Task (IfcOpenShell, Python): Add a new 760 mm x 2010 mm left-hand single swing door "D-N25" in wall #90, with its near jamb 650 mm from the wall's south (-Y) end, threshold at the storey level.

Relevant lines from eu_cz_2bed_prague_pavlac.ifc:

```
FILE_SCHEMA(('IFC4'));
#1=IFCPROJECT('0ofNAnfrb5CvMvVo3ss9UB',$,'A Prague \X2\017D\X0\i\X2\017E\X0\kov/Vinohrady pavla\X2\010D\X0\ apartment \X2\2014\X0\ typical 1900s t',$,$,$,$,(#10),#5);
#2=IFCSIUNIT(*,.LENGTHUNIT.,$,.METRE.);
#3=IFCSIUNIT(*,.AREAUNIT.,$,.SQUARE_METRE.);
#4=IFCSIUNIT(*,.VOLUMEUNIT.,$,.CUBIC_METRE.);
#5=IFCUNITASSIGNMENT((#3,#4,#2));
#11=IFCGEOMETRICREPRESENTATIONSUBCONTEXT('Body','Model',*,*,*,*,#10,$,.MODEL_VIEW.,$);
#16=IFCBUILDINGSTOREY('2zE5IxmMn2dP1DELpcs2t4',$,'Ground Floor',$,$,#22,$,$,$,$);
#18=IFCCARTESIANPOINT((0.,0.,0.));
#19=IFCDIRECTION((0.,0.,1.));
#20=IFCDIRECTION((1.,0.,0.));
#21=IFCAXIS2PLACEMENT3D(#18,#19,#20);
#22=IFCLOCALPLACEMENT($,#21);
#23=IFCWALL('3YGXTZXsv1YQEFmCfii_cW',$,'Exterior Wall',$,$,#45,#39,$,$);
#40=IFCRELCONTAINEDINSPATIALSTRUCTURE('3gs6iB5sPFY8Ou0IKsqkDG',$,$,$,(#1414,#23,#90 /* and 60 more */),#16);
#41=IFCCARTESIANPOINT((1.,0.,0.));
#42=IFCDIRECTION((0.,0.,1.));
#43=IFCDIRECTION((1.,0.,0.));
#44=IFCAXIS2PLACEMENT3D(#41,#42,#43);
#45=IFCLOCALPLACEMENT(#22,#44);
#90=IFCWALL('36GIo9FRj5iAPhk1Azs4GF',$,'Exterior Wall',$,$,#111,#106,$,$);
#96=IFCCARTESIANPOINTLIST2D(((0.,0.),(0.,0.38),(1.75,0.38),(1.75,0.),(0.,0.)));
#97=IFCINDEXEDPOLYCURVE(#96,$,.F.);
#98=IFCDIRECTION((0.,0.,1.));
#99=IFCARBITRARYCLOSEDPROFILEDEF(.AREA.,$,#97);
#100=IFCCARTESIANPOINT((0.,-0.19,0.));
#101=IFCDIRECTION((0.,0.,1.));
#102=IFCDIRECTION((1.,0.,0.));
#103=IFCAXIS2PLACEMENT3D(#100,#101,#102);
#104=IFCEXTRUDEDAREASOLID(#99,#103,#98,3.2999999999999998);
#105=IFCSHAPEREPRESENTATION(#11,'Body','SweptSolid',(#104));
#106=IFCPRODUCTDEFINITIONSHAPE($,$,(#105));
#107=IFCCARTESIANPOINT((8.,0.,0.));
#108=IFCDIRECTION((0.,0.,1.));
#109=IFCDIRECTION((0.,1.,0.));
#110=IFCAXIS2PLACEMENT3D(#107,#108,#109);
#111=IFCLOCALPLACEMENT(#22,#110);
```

```python
import numpy as np
import ifcopenshell
import ifcopenshell.api.feature
import ifcopenshell.api.geometry
import ifcopenshell.api.root
import ifcopenshell.api.spatial
import ifcopenshell.geom
import ifcopenshell.util.element
import ifcopenshell.util.placement
import ifcopenshell.util.representation
import ifcopenshell.util.shape
import ifcopenshell.util.unit

model = ifcopenshell.open("eu_cz_2bed_prague_pavlac.ifc")
unit_scale = ifcopenshell.util.unit.calculate_unit_scale(model)
settings = ifcopenshell.geom.settings()


def volume(element):
    """Net volume in cubic metres, openings subtracted."""
    shape = ifcopenshell.geom.create_shape(settings, element)
    return ifcopenshell.util.shape.get_volume(shape.geometry)


wall = model.by_guid("36GIo9FRj5iAPhk1Azs4GF")
storey = ifcopenshell.util.element.get_container(wall, ifc_class="IfcBuildingStorey")
context = ifcopenshell.util.representation.get_context(model, "Model", "Body", "MODEL_VIEW")
before = volume(wall)

width, height, from_end, sill = 0.76, 2.01, 0.65, 0.0  # metres

# The wall runs along its own X axis, and the end named is its -X end.
wall_shape = ifcopenshell.geom.create_shape(settings, wall)
x, y, z = ifcopenshell.util.shape.get_vertices(wall_shape.geometry).T
start = x.min() + from_end
face, thickness = float(y.min()), float(y.max() - y.min())
wall_matrix = ifcopenshell.util.placement.get_local_placement(wall.ObjectPlacement)
level = ifcopenshell.util.placement.get_local_placement(storey.ObjectPlacement)[2, 3]


def in_wall(x, y):
    """Placement at x, y metres in the wall's axes, at sill height."""
    matrix = wall_matrix.copy()
    matrix[:, 3] = wall_matrix @ np.array([x / unit_scale, y / unit_scale, 0.0, 1.0])
    matrix[2, 3] = level + sill / unit_scale
    return matrix


# Opening: a box that overshoots both wall faces by 50 mm.
opening = ifcopenshell.api.root.create_entity(model, ifc_class="IfcOpeningElement", predefined_type="OPENING")
box = ifcopenshell.api.geometry.add_wall_representation(
    model, context=context, length=width, height=height, thickness=thickness + 0.1
)
ifcopenshell.api.geometry.assign_representation(model, product=opening, representation=box)
ifcopenshell.api.geometry.edit_object_placement(model, product=opening, matrix=in_wall(start, face - 0.05), is_si=False)
ifcopenshell.api.feature.add_feature(model, feature=opening, element=wall)

door = ifcopenshell.api.root.create_entity(model, ifc_class="IfcDoor", name="D-N25", predefined_type="DOOR")
door.OverallWidth, door.OverallHeight = width / unit_scale, height / unit_scale
door.OperationType = "SINGLE_SWING_LEFT"
body = ifcopenshell.api.geometry.add_door_representation(
    model,
    context=context,
    overall_width=door.OverallWidth,
    overall_height=door.OverallHeight,
    operation_type="SINGLE_SWING_LEFT",
    lining_properties={"LiningDepth": thickness / unit_scale, "ThresholdDepth": thickness / unit_scale},
)
ifcopenshell.api.geometry.assign_representation(model, product=door, representation=body)
ifcopenshell.api.spatial.assign_container(model, products=[door], relating_structure=storey)
ifcopenshell.api.feature.add_filling(model, opening=opening, element=door)

# The lining spans the wall, so the door starts at the wall face.
ifcopenshell.api.geometry.edit_object_placement(model, product=door, matrix=in_wall(start, face), is_si=False)

after = volume(wall)

print(f"wall volume {before:.3f} -> {after:.3f} m3")

model.write("eu_cz_2bed_prague_pavlac-out.ifc")
```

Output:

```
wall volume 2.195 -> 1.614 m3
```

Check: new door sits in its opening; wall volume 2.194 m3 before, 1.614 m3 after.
